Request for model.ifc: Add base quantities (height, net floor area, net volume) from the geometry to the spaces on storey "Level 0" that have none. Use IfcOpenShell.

First a look at what the model holds.

```python
import ifcopenshell
import ifcopenshell.util.element
import ifcopenshell.util.unit

model = ifcopenshell.open("model.ifc")
print(model.schema)
for unit_type in ("LENGTHUNIT", "AREAUNIT", "VOLUMEUNIT"):
    print(unit_type, ifcopenshell.util.unit.calculate_unit_scale(model, unit_type))
storey = next(s for s in model.by_type("IfcBuildingStorey") if s.Name == "Level 0")
spaces = [e for e in ifcopenshell.util.element.get_decomposition(storey) if e.is_a("IfcSpace")]
for e in sorted(spaces, key=lambda e: e.id()):
    print(e.id(), e.is_a(), e.Name, list(ifcopenshell.util.element.get_psets(e, qtos_only=True)), sep=" | ")
```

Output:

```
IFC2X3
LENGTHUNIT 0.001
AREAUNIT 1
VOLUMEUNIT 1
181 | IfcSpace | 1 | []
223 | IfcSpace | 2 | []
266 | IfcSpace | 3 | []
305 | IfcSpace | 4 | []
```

```python
import ifcopenshell
import ifcopenshell.api.pset
import ifcopenshell.geom
import ifcopenshell.util.element
import ifcopenshell.util.shape
import ifcopenshell.util.unit

model = ifcopenshell.open("model.ifc")
unit_scale = ifcopenshell.util.unit.calculate_unit_scale(model)
area_scale = ifcopenshell.util.unit.calculate_unit_scale(model, "AREAUNIT")
volume_scale = ifcopenshell.util.unit.calculate_unit_scale(model, "VOLUMEUNIT")
settings = ifcopenshell.geom.settings()

storey = next(s for s in model.by_type("IfcBuildingStorey") if s.Name == "Level 0")
spaces = [e for e in ifcopenshell.util.element.get_decomposition(storey) if e.is_a("IfcSpace")]

for e in sorted(spaces, key=lambda e: e.id()):
    if ifcopenshell.util.element.get_psets(e, qtos_only=True, should_inherit=False):
        continue
    # Geometry comes back in metres, in the element's own axes.
    shape = ifcopenshell.geom.create_shape(settings, e)
    values = {
        "Height": ifcopenshell.util.shape.get_z(shape.geometry) / unit_scale,
        "NetFloorArea": ifcopenshell.util.shape.get_footprint_area(shape.geometry) / area_scale,
        "NetVolume": ifcopenshell.util.shape.get_volume(shape.geometry) / volume_scale,
    }
    qto = ifcopenshell.api.pset.add_qto(model, product=e, name="BaseQuantities")
    ifcopenshell.api.pset.edit_qto(model, qto=qto, properties=values)
    print(e.id(), {k: round(v, 3) for k, v in values.items()})

model.write("model-out.ifc")
```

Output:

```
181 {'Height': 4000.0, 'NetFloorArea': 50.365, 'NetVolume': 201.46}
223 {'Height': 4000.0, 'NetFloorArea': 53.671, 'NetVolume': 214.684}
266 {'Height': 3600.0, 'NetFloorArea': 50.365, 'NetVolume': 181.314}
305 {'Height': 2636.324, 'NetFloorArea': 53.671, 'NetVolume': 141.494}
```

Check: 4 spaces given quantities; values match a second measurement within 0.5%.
